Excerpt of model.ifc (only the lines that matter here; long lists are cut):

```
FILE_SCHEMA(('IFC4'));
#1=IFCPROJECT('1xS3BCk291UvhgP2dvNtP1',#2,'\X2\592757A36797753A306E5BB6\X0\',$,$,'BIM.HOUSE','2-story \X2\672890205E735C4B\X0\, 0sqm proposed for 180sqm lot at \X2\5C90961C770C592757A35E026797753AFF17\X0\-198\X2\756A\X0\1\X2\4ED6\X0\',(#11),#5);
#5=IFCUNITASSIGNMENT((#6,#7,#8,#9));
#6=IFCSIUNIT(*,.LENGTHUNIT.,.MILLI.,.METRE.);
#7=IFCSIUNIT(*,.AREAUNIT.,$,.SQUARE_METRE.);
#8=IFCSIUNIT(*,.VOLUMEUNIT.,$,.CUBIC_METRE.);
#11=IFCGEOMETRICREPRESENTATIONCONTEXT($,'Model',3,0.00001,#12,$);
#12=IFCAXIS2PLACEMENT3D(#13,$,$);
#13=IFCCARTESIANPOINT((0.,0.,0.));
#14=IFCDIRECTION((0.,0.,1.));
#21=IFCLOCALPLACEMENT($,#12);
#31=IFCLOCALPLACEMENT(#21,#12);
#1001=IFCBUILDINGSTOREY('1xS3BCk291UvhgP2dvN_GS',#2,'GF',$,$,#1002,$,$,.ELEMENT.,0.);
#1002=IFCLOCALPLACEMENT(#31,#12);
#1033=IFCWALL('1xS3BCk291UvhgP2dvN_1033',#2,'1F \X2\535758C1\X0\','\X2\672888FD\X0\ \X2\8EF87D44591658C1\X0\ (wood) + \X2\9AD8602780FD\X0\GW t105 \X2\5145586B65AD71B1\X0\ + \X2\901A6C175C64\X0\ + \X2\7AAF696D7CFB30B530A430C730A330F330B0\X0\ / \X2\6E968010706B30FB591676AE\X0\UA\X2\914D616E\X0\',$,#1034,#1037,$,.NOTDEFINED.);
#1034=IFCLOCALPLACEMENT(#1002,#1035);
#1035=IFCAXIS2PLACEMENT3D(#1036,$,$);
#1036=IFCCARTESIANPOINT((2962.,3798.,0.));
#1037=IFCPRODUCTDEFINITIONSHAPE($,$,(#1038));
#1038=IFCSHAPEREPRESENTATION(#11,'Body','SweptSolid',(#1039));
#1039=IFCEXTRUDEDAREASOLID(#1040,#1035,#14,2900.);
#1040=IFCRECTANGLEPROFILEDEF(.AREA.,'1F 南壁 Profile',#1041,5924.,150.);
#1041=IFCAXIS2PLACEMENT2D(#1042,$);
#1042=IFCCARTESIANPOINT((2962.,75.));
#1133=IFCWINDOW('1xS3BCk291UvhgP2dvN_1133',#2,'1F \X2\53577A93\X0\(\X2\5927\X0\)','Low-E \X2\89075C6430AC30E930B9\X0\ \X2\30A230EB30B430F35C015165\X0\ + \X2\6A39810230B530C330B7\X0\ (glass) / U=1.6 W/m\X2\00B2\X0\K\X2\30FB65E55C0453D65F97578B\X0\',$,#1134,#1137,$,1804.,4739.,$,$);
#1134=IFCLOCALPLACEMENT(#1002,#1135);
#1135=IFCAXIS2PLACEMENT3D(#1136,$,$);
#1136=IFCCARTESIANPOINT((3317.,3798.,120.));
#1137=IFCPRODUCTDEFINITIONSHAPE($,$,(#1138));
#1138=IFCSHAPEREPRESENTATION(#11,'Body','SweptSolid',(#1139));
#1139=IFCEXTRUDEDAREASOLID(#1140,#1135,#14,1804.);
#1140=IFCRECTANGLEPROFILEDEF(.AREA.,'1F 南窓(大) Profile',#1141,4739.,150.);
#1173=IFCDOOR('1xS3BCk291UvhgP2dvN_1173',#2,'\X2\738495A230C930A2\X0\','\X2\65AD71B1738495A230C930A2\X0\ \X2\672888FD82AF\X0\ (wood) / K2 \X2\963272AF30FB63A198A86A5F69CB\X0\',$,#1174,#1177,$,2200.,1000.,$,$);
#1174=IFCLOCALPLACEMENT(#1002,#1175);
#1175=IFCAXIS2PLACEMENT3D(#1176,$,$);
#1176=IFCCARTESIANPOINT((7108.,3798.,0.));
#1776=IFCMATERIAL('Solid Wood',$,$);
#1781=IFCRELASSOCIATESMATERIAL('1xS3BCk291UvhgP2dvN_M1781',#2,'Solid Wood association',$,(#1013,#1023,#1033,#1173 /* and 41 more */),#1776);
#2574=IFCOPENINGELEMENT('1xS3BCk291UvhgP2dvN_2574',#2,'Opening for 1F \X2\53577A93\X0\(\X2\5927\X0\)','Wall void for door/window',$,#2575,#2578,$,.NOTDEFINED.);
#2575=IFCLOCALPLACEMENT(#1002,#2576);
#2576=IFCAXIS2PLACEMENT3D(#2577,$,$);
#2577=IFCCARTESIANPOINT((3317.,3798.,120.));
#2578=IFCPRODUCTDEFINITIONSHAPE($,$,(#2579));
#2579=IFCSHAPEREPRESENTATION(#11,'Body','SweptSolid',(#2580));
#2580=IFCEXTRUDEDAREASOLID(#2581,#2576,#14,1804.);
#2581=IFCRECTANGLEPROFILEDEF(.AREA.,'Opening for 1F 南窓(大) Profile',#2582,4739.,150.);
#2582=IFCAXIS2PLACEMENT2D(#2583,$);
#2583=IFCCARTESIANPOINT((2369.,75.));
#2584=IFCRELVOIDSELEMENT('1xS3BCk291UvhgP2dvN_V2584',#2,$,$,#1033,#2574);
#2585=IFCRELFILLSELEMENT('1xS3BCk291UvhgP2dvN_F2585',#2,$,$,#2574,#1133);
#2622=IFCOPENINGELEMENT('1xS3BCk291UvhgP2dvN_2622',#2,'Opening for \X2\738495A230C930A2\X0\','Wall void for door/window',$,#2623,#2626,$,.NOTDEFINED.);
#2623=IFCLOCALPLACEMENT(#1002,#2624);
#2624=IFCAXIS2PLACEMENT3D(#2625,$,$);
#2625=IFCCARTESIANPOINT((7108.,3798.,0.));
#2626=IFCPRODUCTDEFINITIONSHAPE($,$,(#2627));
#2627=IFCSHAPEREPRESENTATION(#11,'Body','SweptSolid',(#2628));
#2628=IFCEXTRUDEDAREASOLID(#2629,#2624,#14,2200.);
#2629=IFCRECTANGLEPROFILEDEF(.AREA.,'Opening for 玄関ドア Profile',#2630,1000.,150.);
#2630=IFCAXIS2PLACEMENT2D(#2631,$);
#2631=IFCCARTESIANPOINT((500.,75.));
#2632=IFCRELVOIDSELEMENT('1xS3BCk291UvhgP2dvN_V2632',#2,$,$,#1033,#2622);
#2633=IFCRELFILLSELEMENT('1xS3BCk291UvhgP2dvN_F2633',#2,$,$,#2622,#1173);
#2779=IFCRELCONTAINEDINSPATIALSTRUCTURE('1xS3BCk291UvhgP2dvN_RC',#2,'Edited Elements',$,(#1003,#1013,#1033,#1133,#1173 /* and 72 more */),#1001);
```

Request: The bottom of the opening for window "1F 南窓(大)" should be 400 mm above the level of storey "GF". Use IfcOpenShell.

```python
import numpy as np
import ifcopenshell
import ifcopenshell.api.geometry
import ifcopenshell.geom
import ifcopenshell.util.element
import ifcopenshell.util.placement
import ifcopenshell.util.shape
import ifcopenshell.util.unit

model = ifcopenshell.open("model.ifc")
unit_scale = ifcopenshell.util.unit.calculate_unit_scale(model)

window = model.by_id(1133)
opening = window.FillsVoids[0].RelatingOpeningElement
storey = ifcopenshell.util.element.get_container(window, ifc_class="IfcBuildingStorey")
level = ifcopenshell.util.placement.get_local_placement(storey.ObjectPlacement)[2, 3]

# The opening's origin need not be at the sill, so measure its lowest point.
shape = ifcopenshell.geom.create_shape(ifcopenshell.geom.settings(), opening)
bottom = ifcopenshell.util.shape.get_shape_bottom_elevation(shape, shape.geometry) / unit_scale
dz = level + 0.4 / unit_scale - bottom

shift = np.array([0.0, 0.0, dz])
# The window is not placed relative to its opening, so move both.
for product in (opening, window):
    matrix = ifcopenshell.util.placement.get_local_placement(product.ObjectPlacement)
    matrix[:3, 3] += shift
    ifcopenshell.api.geometry.edit_object_placement(model, product=product, matrix=matrix, is_si=False)

print(f"moved by {dz * unit_scale:+.3f} m")

model.write("model_edited.ifc")
```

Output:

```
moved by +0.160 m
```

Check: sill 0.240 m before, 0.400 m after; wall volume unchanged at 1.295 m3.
